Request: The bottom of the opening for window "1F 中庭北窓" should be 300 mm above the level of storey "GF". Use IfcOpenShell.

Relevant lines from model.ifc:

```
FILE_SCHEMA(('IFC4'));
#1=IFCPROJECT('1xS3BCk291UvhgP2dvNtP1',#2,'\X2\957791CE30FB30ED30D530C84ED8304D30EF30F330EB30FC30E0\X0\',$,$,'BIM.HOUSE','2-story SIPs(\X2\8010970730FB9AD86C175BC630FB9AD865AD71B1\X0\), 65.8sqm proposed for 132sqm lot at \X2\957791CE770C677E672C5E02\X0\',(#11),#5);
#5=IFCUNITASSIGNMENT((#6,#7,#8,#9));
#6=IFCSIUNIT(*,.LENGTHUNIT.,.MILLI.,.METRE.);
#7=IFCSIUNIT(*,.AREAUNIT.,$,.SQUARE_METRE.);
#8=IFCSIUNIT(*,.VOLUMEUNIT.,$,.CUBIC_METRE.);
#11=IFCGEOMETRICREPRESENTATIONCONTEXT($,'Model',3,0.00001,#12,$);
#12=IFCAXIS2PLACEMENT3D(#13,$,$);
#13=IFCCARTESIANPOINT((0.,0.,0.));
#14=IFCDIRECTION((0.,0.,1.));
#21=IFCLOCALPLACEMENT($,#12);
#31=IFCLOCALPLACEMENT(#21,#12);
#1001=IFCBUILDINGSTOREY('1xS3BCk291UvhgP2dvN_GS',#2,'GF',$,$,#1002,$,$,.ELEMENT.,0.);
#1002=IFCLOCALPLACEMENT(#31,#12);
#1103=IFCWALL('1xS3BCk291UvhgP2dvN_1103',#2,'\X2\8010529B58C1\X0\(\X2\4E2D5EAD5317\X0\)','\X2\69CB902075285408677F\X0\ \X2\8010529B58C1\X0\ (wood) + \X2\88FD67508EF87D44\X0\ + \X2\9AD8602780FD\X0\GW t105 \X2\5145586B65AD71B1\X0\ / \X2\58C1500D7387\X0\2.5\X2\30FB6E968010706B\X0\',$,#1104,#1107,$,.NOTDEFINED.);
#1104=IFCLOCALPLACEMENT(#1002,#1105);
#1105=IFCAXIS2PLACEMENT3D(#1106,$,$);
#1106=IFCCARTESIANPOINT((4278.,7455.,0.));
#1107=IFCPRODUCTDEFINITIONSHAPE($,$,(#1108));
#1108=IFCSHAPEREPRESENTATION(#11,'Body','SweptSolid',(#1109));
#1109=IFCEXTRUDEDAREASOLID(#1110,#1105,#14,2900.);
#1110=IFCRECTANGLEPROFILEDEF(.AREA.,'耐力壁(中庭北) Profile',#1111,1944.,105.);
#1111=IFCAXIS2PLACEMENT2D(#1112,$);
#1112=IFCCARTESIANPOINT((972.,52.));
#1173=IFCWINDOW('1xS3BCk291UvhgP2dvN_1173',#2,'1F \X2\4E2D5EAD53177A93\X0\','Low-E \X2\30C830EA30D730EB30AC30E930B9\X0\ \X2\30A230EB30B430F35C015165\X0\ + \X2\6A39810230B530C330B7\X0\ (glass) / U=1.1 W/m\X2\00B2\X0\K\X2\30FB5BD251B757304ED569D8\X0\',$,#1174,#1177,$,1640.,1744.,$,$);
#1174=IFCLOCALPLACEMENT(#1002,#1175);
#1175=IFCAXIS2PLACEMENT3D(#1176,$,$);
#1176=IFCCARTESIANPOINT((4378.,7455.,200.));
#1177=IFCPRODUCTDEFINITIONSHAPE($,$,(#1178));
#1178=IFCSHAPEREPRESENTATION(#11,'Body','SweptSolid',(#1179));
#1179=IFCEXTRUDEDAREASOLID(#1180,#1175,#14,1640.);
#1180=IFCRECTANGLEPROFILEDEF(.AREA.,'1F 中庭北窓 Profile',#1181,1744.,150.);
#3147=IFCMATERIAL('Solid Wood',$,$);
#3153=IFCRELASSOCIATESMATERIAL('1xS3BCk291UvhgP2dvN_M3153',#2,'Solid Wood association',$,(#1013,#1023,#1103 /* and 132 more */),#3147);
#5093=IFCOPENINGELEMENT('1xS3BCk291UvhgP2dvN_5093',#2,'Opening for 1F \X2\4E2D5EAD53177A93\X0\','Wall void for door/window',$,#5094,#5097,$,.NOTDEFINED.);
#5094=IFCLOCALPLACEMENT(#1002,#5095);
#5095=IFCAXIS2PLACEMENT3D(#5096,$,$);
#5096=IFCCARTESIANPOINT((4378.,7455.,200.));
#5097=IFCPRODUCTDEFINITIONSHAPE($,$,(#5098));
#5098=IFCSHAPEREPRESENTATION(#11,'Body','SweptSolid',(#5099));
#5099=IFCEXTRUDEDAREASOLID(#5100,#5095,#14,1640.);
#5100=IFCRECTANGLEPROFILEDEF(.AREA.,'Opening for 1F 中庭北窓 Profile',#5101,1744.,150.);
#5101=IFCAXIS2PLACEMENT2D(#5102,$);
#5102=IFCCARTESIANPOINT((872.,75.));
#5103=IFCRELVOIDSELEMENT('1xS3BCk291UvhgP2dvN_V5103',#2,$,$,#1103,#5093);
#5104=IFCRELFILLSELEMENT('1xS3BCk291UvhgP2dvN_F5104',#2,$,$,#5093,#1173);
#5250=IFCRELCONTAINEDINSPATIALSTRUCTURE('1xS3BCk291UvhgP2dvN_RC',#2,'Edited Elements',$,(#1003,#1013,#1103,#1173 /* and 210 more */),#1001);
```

```python
import numpy as np
import ifcopenshell
import ifcopenshell.api.geometry
import ifcopenshell.geom
import ifcopenshell.util.element
import ifcopenshell.util.placement
import ifcopenshell.util.shape
import ifcopenshell.util.unit

model = ifcopenshell.open("model.ifc")
unit_scale = ifcopenshell.util.unit.calculate_unit_scale(model)

window = model.by_guid("1xS3BCk291UvhgP2dvN_1173")
opening = window.FillsVoids[0].RelatingOpeningElement
storey = ifcopenshell.util.element.get_container(window, ifc_class="IfcBuildingStorey")
level = ifcopenshell.util.placement.get_local_placement(storey.ObjectPlacement)[2, 3]

# The opening's origin need not be at the sill, so measure its lowest point.
shape = ifcopenshell.geom.create_shape(ifcopenshell.geom.settings(), opening)
bottom = ifcopenshell.util.shape.get_shape_bottom_elevation(shape, shape.geometry) / unit_scale
dz = level + 0.3 / unit_scale - bottom

shift = np.array([0.0, 0.0, dz])
# The window is not placed relative to its opening, so move both.
for product in (opening, window):
    matrix = ifcopenshell.util.placement.get_local_placement(product.ObjectPlacement)
    matrix[:3, 3] += shift
    ifcopenshell.api.geometry.edit_object_placement(model, product=product, matrix=matrix, is_si=False)

print(f"moved by {dz * unit_scale:+.3f} m")

model.write("model-out.ifc")
```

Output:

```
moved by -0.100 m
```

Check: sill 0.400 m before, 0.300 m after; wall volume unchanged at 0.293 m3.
